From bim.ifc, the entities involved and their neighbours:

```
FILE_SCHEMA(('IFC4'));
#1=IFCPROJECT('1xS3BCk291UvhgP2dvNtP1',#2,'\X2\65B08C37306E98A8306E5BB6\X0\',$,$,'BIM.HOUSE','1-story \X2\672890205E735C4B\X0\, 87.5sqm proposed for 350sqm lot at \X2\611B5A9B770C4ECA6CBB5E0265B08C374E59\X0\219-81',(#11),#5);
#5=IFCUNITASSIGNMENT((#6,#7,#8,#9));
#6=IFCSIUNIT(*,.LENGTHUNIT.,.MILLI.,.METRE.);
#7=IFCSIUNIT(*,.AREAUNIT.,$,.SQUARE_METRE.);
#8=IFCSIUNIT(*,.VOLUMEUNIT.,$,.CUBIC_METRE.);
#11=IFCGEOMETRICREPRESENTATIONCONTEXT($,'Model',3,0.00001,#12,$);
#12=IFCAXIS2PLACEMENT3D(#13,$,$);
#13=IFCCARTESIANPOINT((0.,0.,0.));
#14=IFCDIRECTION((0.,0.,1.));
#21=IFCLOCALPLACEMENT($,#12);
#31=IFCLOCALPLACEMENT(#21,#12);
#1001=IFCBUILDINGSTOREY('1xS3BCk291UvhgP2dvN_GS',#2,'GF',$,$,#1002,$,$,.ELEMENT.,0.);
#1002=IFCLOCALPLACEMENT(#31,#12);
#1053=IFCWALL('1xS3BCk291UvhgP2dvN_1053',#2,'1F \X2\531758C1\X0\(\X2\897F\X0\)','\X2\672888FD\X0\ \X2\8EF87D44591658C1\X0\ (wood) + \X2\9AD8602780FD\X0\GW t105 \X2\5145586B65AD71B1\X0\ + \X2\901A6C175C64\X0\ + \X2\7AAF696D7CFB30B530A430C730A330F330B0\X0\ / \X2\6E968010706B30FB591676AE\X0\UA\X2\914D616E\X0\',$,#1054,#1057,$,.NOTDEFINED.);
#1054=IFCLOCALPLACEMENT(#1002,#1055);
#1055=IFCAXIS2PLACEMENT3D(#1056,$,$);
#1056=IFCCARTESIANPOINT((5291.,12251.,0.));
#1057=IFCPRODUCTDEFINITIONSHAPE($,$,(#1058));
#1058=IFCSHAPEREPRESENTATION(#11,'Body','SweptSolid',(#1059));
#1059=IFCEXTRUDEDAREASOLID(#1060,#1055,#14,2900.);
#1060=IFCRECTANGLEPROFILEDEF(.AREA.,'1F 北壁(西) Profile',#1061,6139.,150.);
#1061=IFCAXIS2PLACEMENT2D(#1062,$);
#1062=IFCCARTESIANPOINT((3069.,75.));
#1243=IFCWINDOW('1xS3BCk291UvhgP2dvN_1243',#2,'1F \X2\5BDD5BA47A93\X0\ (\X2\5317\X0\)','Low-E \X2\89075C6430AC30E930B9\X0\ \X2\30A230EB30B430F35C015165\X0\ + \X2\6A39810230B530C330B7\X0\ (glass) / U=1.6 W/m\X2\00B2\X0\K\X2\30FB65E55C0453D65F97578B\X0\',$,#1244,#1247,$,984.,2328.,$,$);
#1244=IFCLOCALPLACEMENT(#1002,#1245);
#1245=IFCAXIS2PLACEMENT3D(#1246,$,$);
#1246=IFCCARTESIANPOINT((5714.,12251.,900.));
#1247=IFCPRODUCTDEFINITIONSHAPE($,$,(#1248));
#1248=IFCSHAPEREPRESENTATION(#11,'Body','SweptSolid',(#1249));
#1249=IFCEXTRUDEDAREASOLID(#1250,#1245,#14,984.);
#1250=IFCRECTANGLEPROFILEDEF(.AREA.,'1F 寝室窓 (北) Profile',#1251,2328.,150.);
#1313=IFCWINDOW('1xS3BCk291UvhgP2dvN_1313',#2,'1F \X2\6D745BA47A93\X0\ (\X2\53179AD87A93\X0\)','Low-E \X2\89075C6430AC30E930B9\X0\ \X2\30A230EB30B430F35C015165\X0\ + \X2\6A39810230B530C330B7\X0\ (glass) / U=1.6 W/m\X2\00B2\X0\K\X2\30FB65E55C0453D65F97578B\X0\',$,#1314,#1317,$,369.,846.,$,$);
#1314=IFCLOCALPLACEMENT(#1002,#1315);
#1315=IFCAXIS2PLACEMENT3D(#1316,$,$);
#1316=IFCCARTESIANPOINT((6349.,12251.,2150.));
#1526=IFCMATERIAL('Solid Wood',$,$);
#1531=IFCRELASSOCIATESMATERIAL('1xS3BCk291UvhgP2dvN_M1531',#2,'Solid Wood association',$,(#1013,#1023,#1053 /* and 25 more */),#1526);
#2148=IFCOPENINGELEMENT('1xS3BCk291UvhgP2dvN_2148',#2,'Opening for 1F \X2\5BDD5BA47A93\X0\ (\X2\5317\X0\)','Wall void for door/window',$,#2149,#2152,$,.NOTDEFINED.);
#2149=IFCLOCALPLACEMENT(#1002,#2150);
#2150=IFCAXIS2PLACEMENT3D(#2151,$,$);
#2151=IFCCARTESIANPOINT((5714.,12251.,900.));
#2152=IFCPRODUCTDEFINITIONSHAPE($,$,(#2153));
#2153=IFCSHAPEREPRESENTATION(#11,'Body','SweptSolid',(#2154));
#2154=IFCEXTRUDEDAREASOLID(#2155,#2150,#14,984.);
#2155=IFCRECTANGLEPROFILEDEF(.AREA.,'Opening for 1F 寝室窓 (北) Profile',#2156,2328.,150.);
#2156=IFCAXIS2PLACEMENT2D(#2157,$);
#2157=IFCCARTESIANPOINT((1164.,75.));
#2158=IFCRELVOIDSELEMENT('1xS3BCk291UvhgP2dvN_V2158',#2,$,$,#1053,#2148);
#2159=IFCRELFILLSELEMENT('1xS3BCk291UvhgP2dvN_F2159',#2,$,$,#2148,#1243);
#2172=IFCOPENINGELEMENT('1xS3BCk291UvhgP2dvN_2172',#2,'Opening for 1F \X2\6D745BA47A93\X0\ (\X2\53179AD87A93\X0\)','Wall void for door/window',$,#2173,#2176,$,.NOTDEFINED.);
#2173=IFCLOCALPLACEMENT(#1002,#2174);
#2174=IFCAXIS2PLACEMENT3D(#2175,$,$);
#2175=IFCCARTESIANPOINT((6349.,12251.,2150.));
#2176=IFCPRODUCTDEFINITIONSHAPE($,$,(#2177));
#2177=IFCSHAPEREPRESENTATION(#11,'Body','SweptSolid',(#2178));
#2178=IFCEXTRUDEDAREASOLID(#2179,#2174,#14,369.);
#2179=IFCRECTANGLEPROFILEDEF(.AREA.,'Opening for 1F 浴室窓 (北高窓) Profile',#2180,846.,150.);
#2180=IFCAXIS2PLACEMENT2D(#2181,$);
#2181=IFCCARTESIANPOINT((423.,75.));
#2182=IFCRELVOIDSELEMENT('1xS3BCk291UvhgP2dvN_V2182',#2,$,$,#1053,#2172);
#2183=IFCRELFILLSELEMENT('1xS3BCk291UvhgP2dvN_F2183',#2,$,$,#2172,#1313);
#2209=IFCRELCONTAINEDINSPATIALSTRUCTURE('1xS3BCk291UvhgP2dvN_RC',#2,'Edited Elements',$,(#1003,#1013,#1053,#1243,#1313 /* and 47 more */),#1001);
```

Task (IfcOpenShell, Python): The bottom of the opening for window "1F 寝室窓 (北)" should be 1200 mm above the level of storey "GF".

```python
import numpy as np
import ifcopenshell
import ifcopenshell.api.geometry
import ifcopenshell.geom
import ifcopenshell.util.element
import ifcopenshell.util.placement
import ifcopenshell.util.shape
import ifcopenshell.util.unit

model = ifcopenshell.open("bim.ifc")
unit_scale = ifcopenshell.util.unit.calculate_unit_scale(model)

window = model.by_guid("1xS3BCk291UvhgP2dvN_1243")
opening = window.FillsVoids[0].RelatingOpeningElement
storey = ifcopenshell.util.element.get_container(window, ifc_class="IfcBuildingStorey")
level = ifcopenshell.util.placement.get_local_placement(storey.ObjectPlacement)[2, 3]

# The opening's origin need not be at the sill, so measure its lowest point.
shape = ifcopenshell.geom.create_shape(ifcopenshell.geom.settings(), opening)
bottom = ifcopenshell.util.shape.get_shape_bottom_elevation(shape, shape.geometry) / unit_scale
dz = level + 1.2 / unit_scale - bottom

shift = np.array([0.0, 0.0, dz])
# The window is not placed relative to its opening, so move both.
for product in (opening, window):
    matrix = ifcopenshell.util.placement.get_local_placement(product.ObjectPlacement)
    matrix[:3, 3] += shift
    ifcopenshell.api.geometry.edit_object_placement(model, product=product, matrix=matrix, is_si=False)

print(f"moved by {dz * unit_scale:+.3f} m")

model.write("bim_updated.ifc")
```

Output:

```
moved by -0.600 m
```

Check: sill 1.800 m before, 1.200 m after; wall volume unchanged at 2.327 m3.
